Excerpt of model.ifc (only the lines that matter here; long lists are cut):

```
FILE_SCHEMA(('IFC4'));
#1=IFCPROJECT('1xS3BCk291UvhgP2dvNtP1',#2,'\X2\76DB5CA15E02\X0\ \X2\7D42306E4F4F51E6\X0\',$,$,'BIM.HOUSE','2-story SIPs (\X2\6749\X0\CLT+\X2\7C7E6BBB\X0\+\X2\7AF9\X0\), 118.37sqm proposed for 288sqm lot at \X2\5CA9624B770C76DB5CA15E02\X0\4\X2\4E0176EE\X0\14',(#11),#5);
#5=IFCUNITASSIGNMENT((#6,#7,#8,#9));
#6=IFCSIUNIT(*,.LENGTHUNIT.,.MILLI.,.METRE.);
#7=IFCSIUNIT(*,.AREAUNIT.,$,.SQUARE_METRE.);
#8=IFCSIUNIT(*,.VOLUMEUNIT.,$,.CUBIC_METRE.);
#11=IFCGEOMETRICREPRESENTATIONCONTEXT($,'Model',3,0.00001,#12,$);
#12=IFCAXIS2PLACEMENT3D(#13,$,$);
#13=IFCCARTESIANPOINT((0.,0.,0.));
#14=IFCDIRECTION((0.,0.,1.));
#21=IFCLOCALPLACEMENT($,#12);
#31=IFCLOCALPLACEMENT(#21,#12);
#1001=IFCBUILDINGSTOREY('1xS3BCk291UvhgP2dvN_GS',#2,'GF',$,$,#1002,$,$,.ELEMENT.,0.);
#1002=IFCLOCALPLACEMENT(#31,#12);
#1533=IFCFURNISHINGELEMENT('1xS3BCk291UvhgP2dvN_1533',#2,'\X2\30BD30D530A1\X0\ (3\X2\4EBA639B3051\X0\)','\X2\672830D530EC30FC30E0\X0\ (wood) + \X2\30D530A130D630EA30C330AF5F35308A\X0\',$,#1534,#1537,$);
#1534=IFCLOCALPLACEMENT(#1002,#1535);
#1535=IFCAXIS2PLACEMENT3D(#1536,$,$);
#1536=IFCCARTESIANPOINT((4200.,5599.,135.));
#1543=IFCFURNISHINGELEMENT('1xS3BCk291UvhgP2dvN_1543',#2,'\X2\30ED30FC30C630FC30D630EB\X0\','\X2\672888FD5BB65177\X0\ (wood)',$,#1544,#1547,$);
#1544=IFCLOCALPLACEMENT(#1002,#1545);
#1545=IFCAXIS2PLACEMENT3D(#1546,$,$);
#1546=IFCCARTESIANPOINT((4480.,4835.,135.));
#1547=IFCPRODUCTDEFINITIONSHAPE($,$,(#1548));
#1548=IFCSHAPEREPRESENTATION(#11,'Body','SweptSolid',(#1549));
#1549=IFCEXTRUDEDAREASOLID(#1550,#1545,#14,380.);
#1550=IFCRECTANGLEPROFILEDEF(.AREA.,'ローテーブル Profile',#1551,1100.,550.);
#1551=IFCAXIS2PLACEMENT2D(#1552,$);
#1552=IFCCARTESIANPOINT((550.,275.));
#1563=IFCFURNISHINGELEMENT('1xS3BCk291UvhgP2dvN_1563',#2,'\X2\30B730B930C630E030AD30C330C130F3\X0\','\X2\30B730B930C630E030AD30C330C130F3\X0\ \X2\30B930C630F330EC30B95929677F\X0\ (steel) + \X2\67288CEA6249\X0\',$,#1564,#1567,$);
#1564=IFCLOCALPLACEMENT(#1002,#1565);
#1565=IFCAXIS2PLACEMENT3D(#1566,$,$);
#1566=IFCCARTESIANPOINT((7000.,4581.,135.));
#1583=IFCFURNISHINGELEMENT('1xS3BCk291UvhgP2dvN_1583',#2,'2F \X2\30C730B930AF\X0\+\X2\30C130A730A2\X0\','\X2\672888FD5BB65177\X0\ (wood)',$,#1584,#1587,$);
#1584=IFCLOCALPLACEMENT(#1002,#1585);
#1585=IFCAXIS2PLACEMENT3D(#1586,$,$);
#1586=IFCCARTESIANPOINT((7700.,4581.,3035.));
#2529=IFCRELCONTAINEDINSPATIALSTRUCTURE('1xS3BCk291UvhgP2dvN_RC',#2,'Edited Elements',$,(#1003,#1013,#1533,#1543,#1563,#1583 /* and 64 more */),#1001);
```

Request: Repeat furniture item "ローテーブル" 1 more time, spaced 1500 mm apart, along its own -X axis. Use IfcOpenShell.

```python
import ifcopenshell
import ifcopenshell.api.geometry
import ifcopenshell.api.root
import ifcopenshell.util.element
import ifcopenshell.util.placement
import ifcopenshell.util.unit

model = ifcopenshell.open("model.ifc")
unit_scale = ifcopenshell.util.unit.calculate_unit_scale(model)


def reuse_history(source, copy):
    """copy_class also copies each property set's owner history, people and application; keep the originals."""
    for rel in copy.IsDefinedBy:
        if rel.is_a("IfcRelDefinesByProperties") and (history := rel.RelatingPropertyDefinition.OwnerHistory):
            rel.RelatingPropertyDefinition.OwnerHistory = source.OwnerHistory
            ifcopenshell.util.element.remove_deep2(model, history)


source = model.by_id(1543)
base = ifcopenshell.util.placement.get_local_placement(source.ObjectPlacement)
step = -base[:3, 0] * 1.5 / unit_scale

for i in range(1, 2):
    copy = ifcopenshell.api.root.copy_class(model, product=source)
    copy.Representation = ifcopenshell.util.element.copy_deep(
        model, source.Representation, exclude=["IfcGeometricRepresentationContext", "IfcRepresentationMap"]
    )
    reuse_history(source, copy)
    matrix = base.copy()
    matrix[:3, 3] += i * step
    print("added at", matrix[:3, 3].round(3) + 0.0)
    ifcopenshell.api.geometry.edit_object_placement(model, product=copy, matrix=matrix, is_si=False)

model.write("model_updated.ifc")
```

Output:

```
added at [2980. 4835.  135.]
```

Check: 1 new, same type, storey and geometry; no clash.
